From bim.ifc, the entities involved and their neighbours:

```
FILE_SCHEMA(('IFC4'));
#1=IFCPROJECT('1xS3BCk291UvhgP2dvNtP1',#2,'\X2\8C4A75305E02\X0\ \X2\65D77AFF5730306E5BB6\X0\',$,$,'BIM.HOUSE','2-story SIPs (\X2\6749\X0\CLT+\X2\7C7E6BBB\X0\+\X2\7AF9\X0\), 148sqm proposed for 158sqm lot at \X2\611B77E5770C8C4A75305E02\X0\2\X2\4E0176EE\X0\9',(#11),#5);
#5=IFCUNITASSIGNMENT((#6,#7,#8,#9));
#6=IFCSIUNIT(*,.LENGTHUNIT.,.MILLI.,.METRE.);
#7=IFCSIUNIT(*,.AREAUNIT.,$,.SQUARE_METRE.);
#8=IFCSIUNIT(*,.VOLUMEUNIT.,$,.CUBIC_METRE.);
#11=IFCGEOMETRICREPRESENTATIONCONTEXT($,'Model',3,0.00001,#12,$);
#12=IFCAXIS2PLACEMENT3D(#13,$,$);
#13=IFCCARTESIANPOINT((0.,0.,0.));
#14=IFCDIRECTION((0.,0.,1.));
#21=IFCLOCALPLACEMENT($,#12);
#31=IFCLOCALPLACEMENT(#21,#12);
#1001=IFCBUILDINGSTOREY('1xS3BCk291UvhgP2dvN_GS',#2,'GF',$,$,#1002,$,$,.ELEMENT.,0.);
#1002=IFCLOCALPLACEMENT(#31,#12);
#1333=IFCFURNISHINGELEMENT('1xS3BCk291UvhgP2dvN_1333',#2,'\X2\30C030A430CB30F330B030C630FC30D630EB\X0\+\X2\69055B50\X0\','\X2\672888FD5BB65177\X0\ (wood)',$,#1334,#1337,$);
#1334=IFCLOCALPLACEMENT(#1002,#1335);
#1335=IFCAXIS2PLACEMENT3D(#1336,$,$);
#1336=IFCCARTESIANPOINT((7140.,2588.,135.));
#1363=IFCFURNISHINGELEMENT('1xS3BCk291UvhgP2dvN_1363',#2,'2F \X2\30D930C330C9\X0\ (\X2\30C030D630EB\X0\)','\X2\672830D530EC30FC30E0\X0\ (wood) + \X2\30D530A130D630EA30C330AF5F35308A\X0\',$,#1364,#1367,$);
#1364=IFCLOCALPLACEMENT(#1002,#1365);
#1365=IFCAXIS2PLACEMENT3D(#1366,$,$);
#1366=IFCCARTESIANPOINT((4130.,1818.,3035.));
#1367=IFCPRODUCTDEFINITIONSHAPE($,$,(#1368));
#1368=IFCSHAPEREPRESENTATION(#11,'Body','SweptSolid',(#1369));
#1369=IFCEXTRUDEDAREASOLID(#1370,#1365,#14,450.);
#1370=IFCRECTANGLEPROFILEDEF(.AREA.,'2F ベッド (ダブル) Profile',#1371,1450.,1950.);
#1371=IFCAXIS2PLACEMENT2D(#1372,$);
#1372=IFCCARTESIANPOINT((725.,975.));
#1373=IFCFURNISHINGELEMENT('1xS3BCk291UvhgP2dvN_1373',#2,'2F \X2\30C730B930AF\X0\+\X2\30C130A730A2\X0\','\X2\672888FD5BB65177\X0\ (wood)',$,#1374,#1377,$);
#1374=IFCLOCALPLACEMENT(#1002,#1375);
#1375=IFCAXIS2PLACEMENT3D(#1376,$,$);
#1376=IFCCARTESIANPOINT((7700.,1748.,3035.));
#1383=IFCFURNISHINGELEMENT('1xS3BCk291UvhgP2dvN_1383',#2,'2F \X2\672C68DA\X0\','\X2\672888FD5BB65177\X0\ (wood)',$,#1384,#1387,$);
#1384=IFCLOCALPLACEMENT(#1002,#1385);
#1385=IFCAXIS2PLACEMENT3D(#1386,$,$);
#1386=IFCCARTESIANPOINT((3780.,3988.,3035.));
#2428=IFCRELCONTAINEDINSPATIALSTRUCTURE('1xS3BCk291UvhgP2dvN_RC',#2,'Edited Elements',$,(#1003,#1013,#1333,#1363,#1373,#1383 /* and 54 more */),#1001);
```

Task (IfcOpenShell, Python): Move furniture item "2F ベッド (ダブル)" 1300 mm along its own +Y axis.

```python
import ifcopenshell
import ifcopenshell.api.geometry
import ifcopenshell.util.placement

model = ifcopenshell.open("bim.ifc")

item = model.by_guid("1xS3BCk291UvhgP2dvN_1363")
matrix = ifcopenshell.util.placement.get_local_placement(item.ObjectPlacement)
matrix[:3, 3] += matrix[:3, 1] * 1300.0
ifcopenshell.api.geometry.edit_object_placement(model, product=item, matrix=matrix, is_si=False)

print(ifcopenshell.util.placement.get_local_placement(item.ObjectPlacement).round(3) + 0.0)

model.write("bim-out.ifc")
```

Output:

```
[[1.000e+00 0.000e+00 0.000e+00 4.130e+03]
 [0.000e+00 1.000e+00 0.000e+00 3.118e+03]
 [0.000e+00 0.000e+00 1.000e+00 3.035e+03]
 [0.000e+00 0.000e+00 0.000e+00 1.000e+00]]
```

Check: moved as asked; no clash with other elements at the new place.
